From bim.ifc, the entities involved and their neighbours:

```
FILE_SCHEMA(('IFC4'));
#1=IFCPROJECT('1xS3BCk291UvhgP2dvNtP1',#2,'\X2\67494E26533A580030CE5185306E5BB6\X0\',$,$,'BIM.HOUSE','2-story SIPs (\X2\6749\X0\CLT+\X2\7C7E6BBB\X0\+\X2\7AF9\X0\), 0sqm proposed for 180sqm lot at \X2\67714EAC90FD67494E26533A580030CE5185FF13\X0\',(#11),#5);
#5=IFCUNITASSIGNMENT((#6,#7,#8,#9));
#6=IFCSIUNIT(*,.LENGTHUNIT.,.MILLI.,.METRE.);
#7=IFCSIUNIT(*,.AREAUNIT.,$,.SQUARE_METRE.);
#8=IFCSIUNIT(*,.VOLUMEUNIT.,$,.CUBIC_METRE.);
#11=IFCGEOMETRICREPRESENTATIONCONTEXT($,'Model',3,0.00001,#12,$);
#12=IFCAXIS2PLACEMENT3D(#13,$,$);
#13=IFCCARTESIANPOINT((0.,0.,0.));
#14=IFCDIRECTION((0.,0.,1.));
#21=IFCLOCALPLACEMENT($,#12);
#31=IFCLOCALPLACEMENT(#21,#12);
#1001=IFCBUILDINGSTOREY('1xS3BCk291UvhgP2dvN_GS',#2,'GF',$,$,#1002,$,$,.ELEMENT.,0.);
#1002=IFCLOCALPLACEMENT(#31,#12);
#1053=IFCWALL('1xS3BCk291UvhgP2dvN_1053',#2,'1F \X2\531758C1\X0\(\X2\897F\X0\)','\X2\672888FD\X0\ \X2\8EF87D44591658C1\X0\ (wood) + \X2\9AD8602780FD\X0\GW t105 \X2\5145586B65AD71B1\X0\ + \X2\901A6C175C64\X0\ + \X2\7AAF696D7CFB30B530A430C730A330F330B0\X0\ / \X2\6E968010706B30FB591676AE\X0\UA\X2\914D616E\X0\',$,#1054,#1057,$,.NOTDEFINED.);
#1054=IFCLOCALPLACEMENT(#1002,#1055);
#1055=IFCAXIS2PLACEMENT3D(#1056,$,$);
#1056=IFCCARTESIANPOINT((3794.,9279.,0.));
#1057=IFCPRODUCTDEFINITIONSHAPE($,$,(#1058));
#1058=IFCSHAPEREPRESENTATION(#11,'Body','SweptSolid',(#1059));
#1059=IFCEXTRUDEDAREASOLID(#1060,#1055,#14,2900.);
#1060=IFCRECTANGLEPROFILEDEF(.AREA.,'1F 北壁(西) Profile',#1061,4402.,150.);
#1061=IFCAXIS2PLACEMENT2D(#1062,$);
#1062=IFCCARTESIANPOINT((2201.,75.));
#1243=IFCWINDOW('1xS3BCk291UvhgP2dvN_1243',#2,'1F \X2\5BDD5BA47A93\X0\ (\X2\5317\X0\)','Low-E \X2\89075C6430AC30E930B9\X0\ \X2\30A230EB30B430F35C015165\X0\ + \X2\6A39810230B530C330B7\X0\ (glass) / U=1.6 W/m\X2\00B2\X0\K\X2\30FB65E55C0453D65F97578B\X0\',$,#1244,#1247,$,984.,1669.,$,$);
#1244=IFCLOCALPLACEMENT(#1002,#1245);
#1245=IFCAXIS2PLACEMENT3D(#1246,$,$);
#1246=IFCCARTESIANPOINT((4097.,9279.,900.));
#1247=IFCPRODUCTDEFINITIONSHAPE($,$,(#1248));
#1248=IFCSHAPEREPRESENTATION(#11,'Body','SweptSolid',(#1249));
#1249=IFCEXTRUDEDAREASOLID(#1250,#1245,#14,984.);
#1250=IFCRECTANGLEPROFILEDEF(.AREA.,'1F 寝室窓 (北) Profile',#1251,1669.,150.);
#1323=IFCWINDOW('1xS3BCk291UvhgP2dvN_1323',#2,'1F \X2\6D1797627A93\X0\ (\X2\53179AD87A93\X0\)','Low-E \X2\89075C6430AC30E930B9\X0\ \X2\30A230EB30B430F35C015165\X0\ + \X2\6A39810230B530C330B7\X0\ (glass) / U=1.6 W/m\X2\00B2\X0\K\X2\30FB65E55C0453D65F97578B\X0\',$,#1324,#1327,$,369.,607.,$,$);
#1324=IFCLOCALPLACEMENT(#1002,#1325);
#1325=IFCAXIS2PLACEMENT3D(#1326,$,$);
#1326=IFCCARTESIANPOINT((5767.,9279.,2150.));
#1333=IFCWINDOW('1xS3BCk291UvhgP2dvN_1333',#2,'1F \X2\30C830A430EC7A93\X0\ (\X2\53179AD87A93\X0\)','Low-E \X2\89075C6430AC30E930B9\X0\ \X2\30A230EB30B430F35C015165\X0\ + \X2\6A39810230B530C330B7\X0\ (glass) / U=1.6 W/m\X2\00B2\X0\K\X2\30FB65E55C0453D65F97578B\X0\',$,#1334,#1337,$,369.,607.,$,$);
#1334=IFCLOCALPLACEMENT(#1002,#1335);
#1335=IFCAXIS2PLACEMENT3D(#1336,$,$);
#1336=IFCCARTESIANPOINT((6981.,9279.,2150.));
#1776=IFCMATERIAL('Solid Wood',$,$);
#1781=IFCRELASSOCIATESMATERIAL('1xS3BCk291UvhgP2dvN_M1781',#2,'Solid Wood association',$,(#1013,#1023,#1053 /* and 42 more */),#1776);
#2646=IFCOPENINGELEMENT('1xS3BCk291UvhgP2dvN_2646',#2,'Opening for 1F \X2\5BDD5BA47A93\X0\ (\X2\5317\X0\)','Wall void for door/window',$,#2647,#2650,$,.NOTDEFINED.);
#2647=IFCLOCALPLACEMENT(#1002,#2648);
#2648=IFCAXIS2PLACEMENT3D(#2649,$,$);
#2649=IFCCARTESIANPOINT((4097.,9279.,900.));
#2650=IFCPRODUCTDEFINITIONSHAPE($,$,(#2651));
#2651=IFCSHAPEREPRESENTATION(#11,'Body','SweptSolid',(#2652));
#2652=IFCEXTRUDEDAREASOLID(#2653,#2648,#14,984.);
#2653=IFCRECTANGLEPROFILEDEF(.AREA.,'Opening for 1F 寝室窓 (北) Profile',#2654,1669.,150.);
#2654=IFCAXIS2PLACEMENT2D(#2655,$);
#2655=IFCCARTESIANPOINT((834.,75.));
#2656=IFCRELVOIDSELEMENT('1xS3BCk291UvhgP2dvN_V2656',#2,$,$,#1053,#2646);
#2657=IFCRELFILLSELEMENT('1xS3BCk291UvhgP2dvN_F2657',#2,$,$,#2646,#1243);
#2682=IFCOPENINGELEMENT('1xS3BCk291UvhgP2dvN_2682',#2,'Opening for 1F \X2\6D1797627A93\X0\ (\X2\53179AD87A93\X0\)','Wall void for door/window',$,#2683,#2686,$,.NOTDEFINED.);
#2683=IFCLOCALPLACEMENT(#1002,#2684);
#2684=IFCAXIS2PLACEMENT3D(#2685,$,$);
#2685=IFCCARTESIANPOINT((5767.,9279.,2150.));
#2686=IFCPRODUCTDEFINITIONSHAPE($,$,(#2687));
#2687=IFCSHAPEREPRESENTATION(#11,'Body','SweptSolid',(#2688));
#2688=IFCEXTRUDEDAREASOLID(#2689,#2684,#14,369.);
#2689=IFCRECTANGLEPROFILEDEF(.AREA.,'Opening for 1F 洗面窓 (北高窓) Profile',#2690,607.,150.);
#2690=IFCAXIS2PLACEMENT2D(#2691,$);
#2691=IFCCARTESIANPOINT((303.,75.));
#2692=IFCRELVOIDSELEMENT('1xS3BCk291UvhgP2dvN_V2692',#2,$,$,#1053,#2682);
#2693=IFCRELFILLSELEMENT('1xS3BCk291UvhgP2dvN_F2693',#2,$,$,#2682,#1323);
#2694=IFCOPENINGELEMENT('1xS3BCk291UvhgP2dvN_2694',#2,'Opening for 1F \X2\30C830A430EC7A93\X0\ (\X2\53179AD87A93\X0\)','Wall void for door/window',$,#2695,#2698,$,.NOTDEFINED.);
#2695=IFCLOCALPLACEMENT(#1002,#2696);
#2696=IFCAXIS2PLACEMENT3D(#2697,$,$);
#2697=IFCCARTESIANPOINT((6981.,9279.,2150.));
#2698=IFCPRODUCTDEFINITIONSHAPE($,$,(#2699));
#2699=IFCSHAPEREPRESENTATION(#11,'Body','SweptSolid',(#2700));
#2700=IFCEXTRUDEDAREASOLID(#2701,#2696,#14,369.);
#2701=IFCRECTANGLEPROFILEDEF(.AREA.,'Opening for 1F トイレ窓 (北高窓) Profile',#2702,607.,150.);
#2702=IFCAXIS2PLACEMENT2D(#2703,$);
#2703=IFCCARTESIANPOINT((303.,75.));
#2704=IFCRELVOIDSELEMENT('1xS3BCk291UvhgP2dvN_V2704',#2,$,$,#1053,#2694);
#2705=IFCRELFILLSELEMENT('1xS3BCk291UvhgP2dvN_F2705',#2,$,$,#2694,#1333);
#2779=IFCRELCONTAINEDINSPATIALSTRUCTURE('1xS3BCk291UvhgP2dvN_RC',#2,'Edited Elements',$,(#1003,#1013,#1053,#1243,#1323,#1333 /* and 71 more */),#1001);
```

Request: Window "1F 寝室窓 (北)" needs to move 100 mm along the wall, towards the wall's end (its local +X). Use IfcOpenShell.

```python
import ifcopenshell
import ifcopenshell.api.geometry
import ifcopenshell.util.placement
import ifcopenshell.util.unit

model = ifcopenshell.open("bim.ifc")
unit_scale = ifcopenshell.util.unit.calculate_unit_scale(model)

window = model.by_id(1243)
opening = window.FillsVoids[0].RelatingOpeningElement
wall = opening.VoidsElements[0].RelatingBuildingElement

wall_matrix = ifcopenshell.util.placement.get_local_placement(wall.ObjectPlacement)
shift = wall_matrix[:3, 0] * 0.1 / unit_scale
before = ifcopenshell.util.placement.get_local_placement(window.ObjectPlacement)[:3, 3].copy()

# The window is not placed relative to its opening, so move both.
for product in (opening, window):
    matrix = ifcopenshell.util.placement.get_local_placement(product.ObjectPlacement)
    matrix[:3, 3] += shift
    ifcopenshell.api.geometry.edit_object_placement(model, product=product, matrix=matrix, is_si=False)

after = ifcopenshell.util.placement.get_local_placement(window.ObjectPlacement)[:3, 3]
print("window moved by", (after - before).round(3) + 0.0)

model.write("bim_edited.ifc")
```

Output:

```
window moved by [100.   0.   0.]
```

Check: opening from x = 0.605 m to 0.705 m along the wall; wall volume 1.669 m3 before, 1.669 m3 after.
